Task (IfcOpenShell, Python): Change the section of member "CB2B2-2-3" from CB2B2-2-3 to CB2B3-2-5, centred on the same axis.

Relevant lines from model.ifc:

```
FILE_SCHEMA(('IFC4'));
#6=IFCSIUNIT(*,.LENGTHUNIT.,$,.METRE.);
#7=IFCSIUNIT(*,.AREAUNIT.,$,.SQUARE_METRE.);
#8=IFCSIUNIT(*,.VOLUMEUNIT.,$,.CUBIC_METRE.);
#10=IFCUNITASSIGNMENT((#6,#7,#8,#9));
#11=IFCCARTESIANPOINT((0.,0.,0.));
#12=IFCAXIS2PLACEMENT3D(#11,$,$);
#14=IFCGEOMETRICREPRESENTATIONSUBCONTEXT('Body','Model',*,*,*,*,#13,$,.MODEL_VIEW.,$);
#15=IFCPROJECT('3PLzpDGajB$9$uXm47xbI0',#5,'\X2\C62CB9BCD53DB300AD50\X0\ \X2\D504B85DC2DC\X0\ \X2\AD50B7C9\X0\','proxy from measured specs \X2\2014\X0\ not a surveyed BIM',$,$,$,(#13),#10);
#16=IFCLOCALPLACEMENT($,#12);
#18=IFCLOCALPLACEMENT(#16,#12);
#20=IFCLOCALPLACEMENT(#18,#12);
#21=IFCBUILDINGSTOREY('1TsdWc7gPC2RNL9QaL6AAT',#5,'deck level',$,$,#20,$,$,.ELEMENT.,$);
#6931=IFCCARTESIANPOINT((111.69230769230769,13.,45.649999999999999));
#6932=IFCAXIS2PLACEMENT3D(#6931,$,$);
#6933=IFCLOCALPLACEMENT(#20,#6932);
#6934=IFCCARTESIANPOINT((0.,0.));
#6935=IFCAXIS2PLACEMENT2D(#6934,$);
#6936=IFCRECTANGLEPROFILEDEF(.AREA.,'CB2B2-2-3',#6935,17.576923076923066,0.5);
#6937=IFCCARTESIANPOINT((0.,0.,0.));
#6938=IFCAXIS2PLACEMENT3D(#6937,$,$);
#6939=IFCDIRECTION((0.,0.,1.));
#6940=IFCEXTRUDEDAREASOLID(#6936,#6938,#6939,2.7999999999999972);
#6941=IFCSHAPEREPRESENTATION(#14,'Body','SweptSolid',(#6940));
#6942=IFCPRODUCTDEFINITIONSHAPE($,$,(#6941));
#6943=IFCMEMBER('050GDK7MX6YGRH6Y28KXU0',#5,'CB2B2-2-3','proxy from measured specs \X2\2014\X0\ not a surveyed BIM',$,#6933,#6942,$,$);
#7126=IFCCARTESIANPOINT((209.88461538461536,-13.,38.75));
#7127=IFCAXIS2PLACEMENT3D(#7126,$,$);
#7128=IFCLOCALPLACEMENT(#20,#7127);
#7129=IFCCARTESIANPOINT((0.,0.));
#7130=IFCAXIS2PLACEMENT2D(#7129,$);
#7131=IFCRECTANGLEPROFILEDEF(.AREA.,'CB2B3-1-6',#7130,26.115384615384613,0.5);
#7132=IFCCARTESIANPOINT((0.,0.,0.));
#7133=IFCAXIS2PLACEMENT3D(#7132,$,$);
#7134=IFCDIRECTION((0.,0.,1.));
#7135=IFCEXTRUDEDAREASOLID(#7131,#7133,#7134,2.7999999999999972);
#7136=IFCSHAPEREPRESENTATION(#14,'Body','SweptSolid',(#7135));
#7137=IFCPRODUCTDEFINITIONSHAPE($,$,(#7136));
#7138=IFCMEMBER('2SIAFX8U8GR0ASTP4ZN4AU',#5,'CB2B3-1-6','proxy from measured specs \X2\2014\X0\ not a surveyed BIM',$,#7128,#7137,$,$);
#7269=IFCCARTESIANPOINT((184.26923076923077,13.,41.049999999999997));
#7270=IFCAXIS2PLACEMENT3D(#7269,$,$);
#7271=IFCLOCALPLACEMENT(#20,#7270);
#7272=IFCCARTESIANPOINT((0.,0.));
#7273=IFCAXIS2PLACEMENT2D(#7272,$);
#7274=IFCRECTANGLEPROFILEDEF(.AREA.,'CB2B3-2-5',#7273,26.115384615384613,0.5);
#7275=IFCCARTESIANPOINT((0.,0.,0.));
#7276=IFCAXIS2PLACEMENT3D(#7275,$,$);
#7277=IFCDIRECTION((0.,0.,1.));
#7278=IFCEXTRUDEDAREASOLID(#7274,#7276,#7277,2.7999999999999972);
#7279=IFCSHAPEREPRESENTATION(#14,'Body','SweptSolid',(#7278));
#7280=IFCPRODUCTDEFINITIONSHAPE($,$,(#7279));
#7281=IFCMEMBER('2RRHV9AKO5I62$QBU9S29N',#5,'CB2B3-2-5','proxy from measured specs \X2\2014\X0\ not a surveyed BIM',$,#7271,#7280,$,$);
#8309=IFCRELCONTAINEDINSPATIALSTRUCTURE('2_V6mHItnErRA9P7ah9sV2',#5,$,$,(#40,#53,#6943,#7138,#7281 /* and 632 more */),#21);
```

```python
import ifcopenshell
import ifcopenshell.util.element
import ifcopenshell.util.representation

model = ifcopenshell.open("model.ifc")

member = model.by_guid("050GDK7MX6YGRH6Y28KXU0")
source = next(p for p in model.by_type("IfcRectangleProfileDef") if p.ProfileName == "CB2B3-2-5")

body = ifcopenshell.util.representation.get_representation(member, "Model", "Body")
solid = body.Items[0]
old_profile = solid.SweptArea

# Copy the section's sizes but keep this member's own profile position.
profile = ifcopenshell.util.element.copy(model, source)
profile.Position = old_profile.Position
solid.SweptArea = profile
if not model.get_total_inverses(old_profile):
    ifcopenshell.util.element.remove_deep2(model, old_profile)
member.Name = member.Name.replace("CB2B2-2-3", "CB2B3-2-5")

print(solid.SweptArea)

model.write("model_v2.ifc")
```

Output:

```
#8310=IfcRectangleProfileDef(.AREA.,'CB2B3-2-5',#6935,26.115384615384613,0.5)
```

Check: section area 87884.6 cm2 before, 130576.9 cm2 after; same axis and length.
